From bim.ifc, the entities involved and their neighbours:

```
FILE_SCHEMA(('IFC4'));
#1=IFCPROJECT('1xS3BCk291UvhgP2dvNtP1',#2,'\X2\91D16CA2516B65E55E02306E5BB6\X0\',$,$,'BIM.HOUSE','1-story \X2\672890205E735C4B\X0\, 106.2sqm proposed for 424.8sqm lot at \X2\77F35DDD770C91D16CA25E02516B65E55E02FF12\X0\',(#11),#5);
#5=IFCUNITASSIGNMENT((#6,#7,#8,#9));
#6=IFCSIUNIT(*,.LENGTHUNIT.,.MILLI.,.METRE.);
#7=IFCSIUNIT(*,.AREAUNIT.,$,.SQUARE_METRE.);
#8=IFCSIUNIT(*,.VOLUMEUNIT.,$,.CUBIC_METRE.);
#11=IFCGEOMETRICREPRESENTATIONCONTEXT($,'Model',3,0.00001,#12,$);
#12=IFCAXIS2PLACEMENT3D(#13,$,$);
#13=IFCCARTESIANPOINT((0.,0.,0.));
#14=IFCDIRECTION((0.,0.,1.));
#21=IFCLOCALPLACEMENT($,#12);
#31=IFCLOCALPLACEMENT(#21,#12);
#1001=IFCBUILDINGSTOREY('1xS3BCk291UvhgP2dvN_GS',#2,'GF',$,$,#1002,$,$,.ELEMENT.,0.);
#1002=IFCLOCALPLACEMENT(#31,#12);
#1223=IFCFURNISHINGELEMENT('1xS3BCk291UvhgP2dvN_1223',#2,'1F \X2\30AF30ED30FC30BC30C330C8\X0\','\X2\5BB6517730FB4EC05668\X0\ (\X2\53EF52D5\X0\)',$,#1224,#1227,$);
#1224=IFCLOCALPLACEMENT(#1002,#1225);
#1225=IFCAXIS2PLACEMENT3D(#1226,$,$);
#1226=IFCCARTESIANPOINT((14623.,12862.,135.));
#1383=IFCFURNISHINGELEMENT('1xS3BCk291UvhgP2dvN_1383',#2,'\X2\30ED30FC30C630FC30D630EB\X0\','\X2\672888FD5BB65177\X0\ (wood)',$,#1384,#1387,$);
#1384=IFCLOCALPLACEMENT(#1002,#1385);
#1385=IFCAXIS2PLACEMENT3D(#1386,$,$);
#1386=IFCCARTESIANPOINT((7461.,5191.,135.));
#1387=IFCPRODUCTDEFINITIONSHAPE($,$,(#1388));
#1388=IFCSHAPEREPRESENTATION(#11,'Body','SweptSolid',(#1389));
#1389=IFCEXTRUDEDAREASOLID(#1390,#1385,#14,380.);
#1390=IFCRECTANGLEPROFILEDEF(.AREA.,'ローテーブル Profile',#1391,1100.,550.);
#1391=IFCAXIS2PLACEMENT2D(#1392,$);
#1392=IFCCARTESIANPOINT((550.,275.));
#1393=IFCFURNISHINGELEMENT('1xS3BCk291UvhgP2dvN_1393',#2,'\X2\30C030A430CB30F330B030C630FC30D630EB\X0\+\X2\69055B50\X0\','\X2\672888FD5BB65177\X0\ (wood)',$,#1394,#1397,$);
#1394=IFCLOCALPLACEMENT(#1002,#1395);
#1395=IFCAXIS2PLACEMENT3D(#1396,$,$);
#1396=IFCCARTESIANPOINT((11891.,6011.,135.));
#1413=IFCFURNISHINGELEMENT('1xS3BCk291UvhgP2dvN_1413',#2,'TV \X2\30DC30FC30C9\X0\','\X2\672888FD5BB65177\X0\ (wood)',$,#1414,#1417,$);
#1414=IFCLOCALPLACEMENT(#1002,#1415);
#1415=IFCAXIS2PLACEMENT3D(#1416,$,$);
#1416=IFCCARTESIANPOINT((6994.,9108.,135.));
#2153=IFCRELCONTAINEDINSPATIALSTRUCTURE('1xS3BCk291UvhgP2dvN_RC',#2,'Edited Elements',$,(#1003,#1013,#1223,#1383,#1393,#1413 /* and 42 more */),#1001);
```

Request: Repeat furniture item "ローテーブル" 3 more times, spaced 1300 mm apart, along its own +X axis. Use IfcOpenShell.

```python
import ifcopenshell
import ifcopenshell.api.geometry
import ifcopenshell.api.root
import ifcopenshell.util.element
import ifcopenshell.util.placement

model = ifcopenshell.open("bim.ifc")


def reuse_history(source, copy):
    """copy_class also copies each property set's owner history, people and application; keep the originals."""
    for rel in copy.IsDefinedBy:
        if rel.is_a("IfcRelDefinesByProperties") and (history := rel.RelatingPropertyDefinition.OwnerHistory):
            rel.RelatingPropertyDefinition.OwnerHistory = source.OwnerHistory
            ifcopenshell.util.element.remove_deep2(model, history)


source = model.by_guid("1xS3BCk291UvhgP2dvN_1383")
base = ifcopenshell.util.placement.get_local_placement(source.ObjectPlacement)
step = base[:3, 0] * 1300.0

for i in range(1, 4):
    copy = ifcopenshell.api.root.copy_class(model, product=source)
    copy.Representation = ifcopenshell.util.element.copy_deep(
        model, source.Representation, exclude=["IfcGeometricRepresentationContext", "IfcRepresentationMap"]
    )
    reuse_history(source, copy)
    matrix = base.copy()
    matrix[:3, 3] += i * step
    print("added at", matrix[:3, 3].round(3) + 0.0)
    ifcopenshell.api.geometry.edit_object_placement(model, product=copy, matrix=matrix, is_si=False)

model.write("bim_edited.ifc")
```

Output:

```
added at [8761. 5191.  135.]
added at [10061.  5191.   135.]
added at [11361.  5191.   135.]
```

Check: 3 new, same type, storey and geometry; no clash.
